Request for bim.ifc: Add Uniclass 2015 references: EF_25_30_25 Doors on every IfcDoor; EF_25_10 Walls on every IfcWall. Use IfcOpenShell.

First a look at what the model holds.

```python
import ifcopenshell

model = ifcopenshell.open("bim.ifc")
print(model.schema)
print("classifications:", [c.Name for c in model.by_type("IfcClassification")])
for ifc_class in ("IfcDoor", "IfcRoof", "IfcStair", "IfcWall", "IfcWindow"):
    print(ifc_class, len(model.by_type(ifc_class)))
```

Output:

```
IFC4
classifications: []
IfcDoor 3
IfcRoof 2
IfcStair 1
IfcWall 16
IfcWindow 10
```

```python
import ifcopenshell
import ifcopenshell.api.classification

model = ifcopenshell.open("bim.ifc")

system = ifcopenshell.api.classification.add_classification(model, classification="Uniclass 2015")

codes = {
    "IfcDoor": ("EF_25_30_25", "Doors"),
    "IfcWall": ("EF_25_10", "Walls"),
}
for ifc_class, (code, name) in codes.items():
    products = model.by_type(ifc_class)
    ifcopenshell.api.classification.add_reference(
        model, products=products, classification=system, identification=code, name=name
    )
    print(code, len(products))

model.write("bim_updated.ifc")
```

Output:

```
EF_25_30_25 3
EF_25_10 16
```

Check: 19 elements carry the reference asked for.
